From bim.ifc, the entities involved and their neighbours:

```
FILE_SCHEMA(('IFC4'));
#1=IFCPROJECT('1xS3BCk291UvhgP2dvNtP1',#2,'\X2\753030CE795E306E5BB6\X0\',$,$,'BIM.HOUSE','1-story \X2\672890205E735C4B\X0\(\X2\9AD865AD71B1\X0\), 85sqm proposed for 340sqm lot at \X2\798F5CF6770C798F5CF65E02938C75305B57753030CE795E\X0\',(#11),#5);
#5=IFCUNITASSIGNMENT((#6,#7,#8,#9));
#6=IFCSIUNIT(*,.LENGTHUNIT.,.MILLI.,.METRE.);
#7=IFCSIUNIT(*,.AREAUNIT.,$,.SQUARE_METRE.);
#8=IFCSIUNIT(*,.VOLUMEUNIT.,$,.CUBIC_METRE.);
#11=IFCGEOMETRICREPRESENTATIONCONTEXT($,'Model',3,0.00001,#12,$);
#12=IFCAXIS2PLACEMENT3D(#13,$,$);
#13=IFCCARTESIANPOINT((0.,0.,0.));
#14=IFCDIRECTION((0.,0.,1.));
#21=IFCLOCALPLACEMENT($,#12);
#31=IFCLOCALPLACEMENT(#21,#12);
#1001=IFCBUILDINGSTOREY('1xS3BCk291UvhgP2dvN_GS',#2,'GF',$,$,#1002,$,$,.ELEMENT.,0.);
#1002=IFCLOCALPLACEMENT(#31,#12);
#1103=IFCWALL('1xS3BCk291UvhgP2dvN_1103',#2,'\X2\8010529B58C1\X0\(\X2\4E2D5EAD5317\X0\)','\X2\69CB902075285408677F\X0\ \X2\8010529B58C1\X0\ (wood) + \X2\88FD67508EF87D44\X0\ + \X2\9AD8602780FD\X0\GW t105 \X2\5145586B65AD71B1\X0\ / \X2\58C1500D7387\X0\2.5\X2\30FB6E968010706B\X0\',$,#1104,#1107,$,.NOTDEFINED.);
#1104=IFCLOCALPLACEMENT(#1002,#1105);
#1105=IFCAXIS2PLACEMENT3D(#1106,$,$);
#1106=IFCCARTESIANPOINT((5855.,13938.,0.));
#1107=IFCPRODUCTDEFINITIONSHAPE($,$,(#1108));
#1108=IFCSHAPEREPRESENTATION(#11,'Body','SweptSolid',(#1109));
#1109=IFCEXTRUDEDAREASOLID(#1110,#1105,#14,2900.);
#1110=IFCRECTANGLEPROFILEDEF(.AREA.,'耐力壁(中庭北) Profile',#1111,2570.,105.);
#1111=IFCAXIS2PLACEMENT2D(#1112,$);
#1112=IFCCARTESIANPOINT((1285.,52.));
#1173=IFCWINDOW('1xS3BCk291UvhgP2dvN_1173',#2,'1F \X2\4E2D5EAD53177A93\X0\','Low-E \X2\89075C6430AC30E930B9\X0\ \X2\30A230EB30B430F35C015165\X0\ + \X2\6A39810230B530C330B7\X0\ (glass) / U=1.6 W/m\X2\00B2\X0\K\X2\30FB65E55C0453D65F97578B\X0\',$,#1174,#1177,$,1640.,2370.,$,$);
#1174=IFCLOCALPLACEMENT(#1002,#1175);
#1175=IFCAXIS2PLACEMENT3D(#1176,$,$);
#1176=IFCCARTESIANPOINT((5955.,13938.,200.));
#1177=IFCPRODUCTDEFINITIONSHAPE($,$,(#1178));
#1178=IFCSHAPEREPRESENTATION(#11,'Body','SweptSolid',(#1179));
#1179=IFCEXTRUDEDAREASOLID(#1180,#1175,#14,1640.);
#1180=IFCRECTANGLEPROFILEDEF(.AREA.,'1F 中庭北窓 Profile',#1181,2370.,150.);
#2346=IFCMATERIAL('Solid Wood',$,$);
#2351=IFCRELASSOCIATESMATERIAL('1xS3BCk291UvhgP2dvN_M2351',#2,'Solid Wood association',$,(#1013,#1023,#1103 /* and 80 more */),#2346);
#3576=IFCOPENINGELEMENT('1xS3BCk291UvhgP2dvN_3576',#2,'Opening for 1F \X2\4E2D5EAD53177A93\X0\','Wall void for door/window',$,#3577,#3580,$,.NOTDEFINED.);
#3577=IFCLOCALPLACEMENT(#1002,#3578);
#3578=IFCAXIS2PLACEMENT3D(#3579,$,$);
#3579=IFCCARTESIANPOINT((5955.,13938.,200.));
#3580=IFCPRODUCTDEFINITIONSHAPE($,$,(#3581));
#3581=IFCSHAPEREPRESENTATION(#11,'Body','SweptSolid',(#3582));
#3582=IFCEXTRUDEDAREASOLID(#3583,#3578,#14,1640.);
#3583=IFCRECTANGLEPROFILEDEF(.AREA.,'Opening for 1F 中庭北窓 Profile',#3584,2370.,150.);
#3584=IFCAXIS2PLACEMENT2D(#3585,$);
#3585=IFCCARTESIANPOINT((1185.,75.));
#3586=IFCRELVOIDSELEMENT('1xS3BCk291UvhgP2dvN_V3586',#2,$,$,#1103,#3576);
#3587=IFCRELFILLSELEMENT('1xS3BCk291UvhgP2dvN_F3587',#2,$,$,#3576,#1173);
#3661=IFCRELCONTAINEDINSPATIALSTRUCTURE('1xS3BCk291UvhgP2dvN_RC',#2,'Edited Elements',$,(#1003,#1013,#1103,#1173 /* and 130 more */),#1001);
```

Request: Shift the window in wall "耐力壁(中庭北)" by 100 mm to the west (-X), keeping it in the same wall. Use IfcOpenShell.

```python
import ifcopenshell
import ifcopenshell.api.geometry
import ifcopenshell.util.placement
import ifcopenshell.util.unit

model = ifcopenshell.open("bim.ifc")
unit_scale = ifcopenshell.util.unit.calculate_unit_scale(model)

window = model.by_guid("1xS3BCk291UvhgP2dvN_1173")
opening = window.FillsVoids[0].RelatingOpeningElement
wall = opening.VoidsElements[0].RelatingBuildingElement

wall_matrix = ifcopenshell.util.placement.get_local_placement(wall.ObjectPlacement)
shift = wall_matrix[:3, 0] * -0.1 / unit_scale
before = ifcopenshell.util.placement.get_local_placement(window.ObjectPlacement)[:3, 3].copy()

# The window is not placed relative to its opening, so move both.
for product in (opening, window):
    matrix = ifcopenshell.util.placement.get_local_placement(product.ObjectPlacement)
    matrix[:3, 3] += shift
    ifcopenshell.api.geometry.edit_object_placement(model, product=product, matrix=matrix, is_si=False)

after = ifcopenshell.util.placement.get_local_placement(window.ObjectPlacement)[:3, 3]
print("window moved by", (after - before).round(3) + 0.0)

model.write("bim-out.ifc")
```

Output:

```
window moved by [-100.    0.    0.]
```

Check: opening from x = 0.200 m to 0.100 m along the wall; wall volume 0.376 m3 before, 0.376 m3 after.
